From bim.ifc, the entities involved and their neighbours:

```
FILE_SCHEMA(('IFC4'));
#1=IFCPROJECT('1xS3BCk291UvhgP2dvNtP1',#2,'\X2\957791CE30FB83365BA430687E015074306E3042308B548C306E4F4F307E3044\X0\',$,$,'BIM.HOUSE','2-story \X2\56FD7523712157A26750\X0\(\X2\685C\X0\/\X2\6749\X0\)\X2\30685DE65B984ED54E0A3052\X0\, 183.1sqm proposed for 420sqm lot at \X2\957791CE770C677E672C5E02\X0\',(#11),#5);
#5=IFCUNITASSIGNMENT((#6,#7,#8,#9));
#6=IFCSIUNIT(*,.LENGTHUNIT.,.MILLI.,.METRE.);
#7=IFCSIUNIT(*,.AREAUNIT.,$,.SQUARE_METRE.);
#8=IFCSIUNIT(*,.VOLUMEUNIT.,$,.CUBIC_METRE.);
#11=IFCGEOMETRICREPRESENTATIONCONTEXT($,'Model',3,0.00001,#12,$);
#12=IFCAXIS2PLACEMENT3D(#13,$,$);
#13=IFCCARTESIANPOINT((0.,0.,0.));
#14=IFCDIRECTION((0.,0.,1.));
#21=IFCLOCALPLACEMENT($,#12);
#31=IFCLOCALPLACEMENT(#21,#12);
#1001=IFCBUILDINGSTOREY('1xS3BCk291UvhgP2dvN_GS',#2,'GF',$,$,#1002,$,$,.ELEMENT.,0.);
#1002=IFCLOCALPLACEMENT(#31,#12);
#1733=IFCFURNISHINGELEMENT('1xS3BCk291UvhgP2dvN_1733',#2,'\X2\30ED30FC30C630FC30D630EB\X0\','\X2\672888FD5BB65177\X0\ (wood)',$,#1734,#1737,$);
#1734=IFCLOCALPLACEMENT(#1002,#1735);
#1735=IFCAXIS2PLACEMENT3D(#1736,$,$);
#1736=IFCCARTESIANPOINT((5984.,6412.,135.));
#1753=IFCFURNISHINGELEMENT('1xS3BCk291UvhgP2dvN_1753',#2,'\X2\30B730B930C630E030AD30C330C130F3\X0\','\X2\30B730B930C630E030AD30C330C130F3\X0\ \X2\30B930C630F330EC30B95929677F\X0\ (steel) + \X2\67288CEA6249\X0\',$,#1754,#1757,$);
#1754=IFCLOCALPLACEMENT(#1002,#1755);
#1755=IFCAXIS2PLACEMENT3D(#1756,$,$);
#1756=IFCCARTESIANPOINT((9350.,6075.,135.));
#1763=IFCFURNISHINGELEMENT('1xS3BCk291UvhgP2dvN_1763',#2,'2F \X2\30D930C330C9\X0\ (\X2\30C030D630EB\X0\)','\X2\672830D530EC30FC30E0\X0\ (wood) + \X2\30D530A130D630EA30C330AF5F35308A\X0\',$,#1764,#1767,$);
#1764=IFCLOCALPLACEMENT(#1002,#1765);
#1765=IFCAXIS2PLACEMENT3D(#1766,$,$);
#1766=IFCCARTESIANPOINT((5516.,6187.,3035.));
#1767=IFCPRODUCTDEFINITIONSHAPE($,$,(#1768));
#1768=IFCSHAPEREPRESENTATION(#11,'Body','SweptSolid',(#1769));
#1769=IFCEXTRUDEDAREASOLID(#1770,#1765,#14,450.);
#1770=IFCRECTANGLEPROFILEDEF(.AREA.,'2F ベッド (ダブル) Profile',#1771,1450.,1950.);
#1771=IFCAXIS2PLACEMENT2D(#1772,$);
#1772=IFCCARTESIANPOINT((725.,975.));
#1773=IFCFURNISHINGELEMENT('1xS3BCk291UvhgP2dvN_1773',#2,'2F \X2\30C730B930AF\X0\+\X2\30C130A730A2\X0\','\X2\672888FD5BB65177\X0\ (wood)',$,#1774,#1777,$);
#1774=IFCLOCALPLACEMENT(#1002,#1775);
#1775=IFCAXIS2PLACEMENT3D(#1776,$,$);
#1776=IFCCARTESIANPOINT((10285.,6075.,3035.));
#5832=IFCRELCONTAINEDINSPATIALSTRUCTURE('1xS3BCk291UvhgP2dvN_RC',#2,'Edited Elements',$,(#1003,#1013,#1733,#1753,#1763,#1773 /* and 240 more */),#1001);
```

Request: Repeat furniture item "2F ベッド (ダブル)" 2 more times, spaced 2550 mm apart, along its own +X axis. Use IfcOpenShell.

```python
import ifcopenshell
import ifcopenshell.api.geometry
import ifcopenshell.api.root
import ifcopenshell.util.element
import ifcopenshell.util.placement
import ifcopenshell.util.unit

model = ifcopenshell.open("bim.ifc")
unit_scale = ifcopenshell.util.unit.calculate_unit_scale(model)


def reuse_history(source, copy):
    """copy_class also copies each property set's owner history, people and application; keep the originals."""
    for rel in copy.IsDefinedBy:
        if rel.is_a("IfcRelDefinesByProperties") and (history := rel.RelatingPropertyDefinition.OwnerHistory):
            rel.RelatingPropertyDefinition.OwnerHistory = source.OwnerHistory
            ifcopenshell.util.element.remove_deep2(model, history)


source = model.by_id(1763)
base = ifcopenshell.util.placement.get_local_placement(source.ObjectPlacement)
step = base[:3, 0] * 2.55 / unit_scale

for i in range(1, 3):
    copy = ifcopenshell.api.root.copy_class(model, product=source)
    copy.Representation = ifcopenshell.util.element.copy_deep(
        model, source.Representation, exclude=["IfcGeometricRepresentationContext", "IfcRepresentationMap"]
    )
    reuse_history(source, copy)
    matrix = base.copy()
    matrix[:3, 3] += i * step
    print("added at", matrix[:3, 3].round(3) + 0.0)
    ifcopenshell.api.geometry.edit_object_placement(model, product=copy, matrix=matrix, is_si=False)

model.write("bim_rev.ifc")
```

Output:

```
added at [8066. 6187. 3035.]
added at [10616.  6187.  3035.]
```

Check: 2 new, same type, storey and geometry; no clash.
